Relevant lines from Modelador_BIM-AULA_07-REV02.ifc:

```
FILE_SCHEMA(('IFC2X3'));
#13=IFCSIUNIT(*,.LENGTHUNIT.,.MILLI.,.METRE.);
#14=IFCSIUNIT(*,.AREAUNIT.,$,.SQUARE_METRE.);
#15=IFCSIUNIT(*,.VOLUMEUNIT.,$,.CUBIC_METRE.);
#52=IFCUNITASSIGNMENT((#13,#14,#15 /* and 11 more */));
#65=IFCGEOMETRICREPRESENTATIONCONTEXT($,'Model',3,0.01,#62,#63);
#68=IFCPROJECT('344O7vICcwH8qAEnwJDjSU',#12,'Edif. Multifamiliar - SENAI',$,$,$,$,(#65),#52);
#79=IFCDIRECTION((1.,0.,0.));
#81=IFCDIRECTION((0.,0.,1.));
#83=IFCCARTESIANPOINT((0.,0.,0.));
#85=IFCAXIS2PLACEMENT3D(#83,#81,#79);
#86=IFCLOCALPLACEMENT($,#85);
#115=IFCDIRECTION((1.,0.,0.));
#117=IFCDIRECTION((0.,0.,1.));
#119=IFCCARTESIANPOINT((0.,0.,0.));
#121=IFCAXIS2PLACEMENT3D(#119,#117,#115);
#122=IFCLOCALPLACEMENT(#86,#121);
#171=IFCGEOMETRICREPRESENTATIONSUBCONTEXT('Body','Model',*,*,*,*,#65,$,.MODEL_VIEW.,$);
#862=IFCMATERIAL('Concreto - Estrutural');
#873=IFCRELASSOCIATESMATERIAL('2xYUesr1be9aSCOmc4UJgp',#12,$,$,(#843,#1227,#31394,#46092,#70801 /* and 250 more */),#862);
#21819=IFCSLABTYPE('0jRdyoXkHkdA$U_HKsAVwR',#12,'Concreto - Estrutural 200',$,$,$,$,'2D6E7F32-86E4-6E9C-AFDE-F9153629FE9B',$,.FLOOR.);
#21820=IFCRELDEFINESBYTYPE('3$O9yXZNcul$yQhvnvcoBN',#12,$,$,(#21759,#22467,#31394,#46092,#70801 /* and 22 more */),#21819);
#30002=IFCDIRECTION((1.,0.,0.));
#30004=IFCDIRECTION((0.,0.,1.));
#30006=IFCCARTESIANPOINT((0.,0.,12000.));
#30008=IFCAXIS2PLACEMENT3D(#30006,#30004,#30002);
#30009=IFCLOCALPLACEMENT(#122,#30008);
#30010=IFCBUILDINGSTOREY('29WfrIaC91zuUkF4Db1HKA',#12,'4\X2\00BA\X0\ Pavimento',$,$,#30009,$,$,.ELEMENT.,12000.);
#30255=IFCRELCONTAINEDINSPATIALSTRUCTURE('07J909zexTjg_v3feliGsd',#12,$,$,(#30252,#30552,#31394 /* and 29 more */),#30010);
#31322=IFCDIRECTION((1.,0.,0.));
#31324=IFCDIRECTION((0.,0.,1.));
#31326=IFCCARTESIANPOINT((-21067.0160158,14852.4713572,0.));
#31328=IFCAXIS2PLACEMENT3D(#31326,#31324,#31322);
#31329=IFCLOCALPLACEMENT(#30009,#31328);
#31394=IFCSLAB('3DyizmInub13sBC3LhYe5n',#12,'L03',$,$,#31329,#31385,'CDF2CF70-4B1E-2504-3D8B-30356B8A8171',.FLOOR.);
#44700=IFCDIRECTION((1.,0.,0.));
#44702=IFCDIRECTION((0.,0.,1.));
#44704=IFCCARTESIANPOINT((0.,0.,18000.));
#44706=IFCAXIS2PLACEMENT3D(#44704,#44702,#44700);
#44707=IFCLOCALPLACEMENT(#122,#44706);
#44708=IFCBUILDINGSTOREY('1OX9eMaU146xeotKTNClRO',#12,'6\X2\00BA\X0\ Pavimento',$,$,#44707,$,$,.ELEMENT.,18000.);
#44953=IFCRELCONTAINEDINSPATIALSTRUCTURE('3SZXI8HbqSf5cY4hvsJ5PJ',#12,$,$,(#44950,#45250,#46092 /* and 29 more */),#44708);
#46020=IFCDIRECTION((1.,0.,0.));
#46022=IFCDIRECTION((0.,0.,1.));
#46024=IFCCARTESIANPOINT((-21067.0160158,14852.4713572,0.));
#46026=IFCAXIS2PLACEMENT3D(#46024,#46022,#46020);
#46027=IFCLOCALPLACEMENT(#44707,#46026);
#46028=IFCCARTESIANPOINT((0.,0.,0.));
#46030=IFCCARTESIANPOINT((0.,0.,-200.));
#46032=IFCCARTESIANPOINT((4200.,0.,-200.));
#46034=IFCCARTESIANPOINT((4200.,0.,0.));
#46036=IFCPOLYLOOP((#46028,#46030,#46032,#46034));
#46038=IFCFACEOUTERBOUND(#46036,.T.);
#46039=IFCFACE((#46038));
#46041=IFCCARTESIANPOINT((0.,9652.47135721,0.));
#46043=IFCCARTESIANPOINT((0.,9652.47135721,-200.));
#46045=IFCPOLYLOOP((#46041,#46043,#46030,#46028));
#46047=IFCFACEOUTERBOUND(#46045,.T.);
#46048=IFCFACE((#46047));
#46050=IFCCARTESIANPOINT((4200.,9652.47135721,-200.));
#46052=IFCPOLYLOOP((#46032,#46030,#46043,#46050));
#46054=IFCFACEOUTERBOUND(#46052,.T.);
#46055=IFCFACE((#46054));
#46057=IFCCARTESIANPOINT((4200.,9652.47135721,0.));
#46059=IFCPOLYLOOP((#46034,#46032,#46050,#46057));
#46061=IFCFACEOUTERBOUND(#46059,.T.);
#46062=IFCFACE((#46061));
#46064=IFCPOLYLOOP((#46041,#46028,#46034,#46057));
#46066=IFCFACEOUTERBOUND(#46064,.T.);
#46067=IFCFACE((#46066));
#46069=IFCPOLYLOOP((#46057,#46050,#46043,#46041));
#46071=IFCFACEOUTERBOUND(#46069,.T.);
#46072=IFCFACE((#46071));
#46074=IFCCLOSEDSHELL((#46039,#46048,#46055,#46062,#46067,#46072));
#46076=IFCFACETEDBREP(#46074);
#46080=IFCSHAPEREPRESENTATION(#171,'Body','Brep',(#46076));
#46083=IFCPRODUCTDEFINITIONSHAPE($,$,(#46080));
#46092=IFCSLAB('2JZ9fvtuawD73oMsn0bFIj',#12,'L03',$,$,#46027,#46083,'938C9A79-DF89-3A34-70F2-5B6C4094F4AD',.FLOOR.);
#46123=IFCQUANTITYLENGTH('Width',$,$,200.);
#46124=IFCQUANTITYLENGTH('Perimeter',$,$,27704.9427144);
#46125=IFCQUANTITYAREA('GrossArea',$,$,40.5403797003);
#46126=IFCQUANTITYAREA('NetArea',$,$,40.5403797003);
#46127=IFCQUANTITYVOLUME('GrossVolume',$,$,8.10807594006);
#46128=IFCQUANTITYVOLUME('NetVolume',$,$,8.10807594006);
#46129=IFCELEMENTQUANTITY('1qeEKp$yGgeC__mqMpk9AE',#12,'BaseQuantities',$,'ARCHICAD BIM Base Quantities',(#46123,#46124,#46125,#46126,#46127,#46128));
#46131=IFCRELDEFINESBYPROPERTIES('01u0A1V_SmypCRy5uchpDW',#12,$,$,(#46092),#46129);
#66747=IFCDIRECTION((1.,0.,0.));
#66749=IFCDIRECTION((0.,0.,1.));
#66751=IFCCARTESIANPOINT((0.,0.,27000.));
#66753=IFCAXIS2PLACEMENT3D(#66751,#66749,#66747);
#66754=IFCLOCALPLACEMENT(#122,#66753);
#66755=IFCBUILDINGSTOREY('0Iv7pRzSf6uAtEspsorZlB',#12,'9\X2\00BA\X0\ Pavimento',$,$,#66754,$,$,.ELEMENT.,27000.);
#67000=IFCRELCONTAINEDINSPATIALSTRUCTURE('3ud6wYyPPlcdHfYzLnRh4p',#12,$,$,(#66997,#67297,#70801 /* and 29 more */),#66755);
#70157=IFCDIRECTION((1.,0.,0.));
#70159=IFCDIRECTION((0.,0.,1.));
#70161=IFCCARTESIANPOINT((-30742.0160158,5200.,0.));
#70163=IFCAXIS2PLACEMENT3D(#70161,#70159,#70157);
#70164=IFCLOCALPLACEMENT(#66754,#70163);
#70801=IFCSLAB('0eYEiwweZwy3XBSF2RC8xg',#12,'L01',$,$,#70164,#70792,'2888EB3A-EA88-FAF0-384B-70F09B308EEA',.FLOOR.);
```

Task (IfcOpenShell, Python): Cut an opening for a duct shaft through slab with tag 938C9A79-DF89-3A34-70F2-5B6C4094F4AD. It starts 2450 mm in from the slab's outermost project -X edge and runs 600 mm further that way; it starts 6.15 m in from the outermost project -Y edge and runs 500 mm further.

```python
import numpy as np
import ifcopenshell
import ifcopenshell.api.feature
import ifcopenshell.api.geometry
import ifcopenshell.api.pset
import ifcopenshell.api.root
import ifcopenshell.geom
import ifcopenshell.util.element
import ifcopenshell.util.placement
import ifcopenshell.util.representation
import ifcopenshell.util.shape
import ifcopenshell.util.unit

model = ifcopenshell.open("Modelador_BIM-AULA_07-REV02.ifc")
unit_scale = ifcopenshell.util.unit.calculate_unit_scale(model)
area_scale = ifcopenshell.util.unit.calculate_unit_scale(model, "AREAUNIT")
volume_scale = ifcopenshell.util.unit.calculate_unit_scale(model, "VOLUMEUNIT")
settings = ifcopenshell.geom.settings()


def volume(element):
    """Net volume in cubic metres, openings subtracted."""
    shape = ifcopenshell.geom.create_shape(settings, element)
    return ifcopenshell.util.shape.get_volume(shape.geometry)


slab = model.by_id(46092)
before = volume(slab)

# Extent in the slab's own axes, in metres. The edges named are its -X and -Y sides.
slab_shape = ifcopenshell.geom.create_shape(settings, slab)
vertices = ifcopenshell.util.shape.get_vertices(slab_shape.geometry)
x_min, y_min, bottom = vertices.min(axis=0)
top = vertices[:, 2].max()

opening = ifcopenshell.api.root.create_entity(model, ifc_class="IfcOpeningElement", name="Duct shaft opening")
context = ifcopenshell.util.representation.get_context(model, "Model", "Body", "MODEL_VIEW")
width, depth = 0.6, 0.5
outline = [(0.0, 0.0), (width, 0.0), (width, depth), (0.0, depth), (0.0, 0.0)]
# Overshoot both faces by 50 mm so the cut is clean.
shape = ifcopenshell.api.geometry.add_slab_representation(
    model, context=context, depth=top - bottom + 0.1, polyline=outline
)
ifcopenshell.api.geometry.assign_representation(model, product=opening, representation=shape)

matrix = ifcopenshell.util.placement.get_local_placement(slab.ObjectPlacement)
matrix[:, 3] = matrix @ np.append(np.array([x_min + 2.45, y_min + 6.15, bottom - 0.05]) / unit_scale, 1.0)
ifcopenshell.api.geometry.edit_object_placement(model, product=opening, matrix=matrix, is_si=False)
ifcopenshell.api.feature.add_feature(model, feature=opening, element=slab)

after = volume(slab)

# Update the slab's stored quantities.
qto = model.by_id(ifcopenshell.util.element.get_pset(slab, "BaseQuantities", should_inherit=False)["id"])
ifcopenshell.api.pset.edit_qto(model, qto=qto, properties={
    "NetArea": after / (top - bottom) / area_scale,
    "NetVolume": after / volume_scale,
})

print(f"slab volume {before:.3f} -> {after:.3f} m3")

model.write("Modelador_BIM-AULA_07-REV02_updated.ifc")
```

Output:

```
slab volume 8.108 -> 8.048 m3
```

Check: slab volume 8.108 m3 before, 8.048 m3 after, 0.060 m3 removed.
